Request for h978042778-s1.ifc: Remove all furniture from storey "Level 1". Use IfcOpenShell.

First a look at what the model holds.

```python
import ifcopenshell
import ifcopenshell.util.element

model = ifcopenshell.open("h978042778-s1.ifc")
print(model.schema)
storey = next(s for s in model.by_type("IfcBuildingStorey") if s.Name == "Level 1")
furniture = [e for e in ifcopenshell.util.element.get_decomposition(storey) if e.is_a("IfcFurnishingElement")]
seen = {}
for e in furniture:
    element_type = ifcopenshell.util.element.get_type(e)
    name = element_type.Name if element_type not in (None, e) else None
    seen[name] = seen.get(name, 0) + 1
for name, count in sorted(seen.items(), key=str):
    print(count, "x", name)
```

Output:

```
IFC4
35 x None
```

```python
import ifcopenshell
import ifcopenshell.api.root
import ifcopenshell.util.element

model = ifcopenshell.open("h978042778-s1.ifc")

storey = next(s for s in model.by_type("IfcBuildingStorey") if s.Name == "Level 1")
furniture = [e for e in ifcopenshell.util.element.get_decomposition(storey) if e.is_a("IfcFurnishingElement")]

for e in furniture:
    ifcopenshell.api.root.remove_product(model, product=e)
print(len(furniture), "removed")

model.write("h978042778-s1-out.ifc")
```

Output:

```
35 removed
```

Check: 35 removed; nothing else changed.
